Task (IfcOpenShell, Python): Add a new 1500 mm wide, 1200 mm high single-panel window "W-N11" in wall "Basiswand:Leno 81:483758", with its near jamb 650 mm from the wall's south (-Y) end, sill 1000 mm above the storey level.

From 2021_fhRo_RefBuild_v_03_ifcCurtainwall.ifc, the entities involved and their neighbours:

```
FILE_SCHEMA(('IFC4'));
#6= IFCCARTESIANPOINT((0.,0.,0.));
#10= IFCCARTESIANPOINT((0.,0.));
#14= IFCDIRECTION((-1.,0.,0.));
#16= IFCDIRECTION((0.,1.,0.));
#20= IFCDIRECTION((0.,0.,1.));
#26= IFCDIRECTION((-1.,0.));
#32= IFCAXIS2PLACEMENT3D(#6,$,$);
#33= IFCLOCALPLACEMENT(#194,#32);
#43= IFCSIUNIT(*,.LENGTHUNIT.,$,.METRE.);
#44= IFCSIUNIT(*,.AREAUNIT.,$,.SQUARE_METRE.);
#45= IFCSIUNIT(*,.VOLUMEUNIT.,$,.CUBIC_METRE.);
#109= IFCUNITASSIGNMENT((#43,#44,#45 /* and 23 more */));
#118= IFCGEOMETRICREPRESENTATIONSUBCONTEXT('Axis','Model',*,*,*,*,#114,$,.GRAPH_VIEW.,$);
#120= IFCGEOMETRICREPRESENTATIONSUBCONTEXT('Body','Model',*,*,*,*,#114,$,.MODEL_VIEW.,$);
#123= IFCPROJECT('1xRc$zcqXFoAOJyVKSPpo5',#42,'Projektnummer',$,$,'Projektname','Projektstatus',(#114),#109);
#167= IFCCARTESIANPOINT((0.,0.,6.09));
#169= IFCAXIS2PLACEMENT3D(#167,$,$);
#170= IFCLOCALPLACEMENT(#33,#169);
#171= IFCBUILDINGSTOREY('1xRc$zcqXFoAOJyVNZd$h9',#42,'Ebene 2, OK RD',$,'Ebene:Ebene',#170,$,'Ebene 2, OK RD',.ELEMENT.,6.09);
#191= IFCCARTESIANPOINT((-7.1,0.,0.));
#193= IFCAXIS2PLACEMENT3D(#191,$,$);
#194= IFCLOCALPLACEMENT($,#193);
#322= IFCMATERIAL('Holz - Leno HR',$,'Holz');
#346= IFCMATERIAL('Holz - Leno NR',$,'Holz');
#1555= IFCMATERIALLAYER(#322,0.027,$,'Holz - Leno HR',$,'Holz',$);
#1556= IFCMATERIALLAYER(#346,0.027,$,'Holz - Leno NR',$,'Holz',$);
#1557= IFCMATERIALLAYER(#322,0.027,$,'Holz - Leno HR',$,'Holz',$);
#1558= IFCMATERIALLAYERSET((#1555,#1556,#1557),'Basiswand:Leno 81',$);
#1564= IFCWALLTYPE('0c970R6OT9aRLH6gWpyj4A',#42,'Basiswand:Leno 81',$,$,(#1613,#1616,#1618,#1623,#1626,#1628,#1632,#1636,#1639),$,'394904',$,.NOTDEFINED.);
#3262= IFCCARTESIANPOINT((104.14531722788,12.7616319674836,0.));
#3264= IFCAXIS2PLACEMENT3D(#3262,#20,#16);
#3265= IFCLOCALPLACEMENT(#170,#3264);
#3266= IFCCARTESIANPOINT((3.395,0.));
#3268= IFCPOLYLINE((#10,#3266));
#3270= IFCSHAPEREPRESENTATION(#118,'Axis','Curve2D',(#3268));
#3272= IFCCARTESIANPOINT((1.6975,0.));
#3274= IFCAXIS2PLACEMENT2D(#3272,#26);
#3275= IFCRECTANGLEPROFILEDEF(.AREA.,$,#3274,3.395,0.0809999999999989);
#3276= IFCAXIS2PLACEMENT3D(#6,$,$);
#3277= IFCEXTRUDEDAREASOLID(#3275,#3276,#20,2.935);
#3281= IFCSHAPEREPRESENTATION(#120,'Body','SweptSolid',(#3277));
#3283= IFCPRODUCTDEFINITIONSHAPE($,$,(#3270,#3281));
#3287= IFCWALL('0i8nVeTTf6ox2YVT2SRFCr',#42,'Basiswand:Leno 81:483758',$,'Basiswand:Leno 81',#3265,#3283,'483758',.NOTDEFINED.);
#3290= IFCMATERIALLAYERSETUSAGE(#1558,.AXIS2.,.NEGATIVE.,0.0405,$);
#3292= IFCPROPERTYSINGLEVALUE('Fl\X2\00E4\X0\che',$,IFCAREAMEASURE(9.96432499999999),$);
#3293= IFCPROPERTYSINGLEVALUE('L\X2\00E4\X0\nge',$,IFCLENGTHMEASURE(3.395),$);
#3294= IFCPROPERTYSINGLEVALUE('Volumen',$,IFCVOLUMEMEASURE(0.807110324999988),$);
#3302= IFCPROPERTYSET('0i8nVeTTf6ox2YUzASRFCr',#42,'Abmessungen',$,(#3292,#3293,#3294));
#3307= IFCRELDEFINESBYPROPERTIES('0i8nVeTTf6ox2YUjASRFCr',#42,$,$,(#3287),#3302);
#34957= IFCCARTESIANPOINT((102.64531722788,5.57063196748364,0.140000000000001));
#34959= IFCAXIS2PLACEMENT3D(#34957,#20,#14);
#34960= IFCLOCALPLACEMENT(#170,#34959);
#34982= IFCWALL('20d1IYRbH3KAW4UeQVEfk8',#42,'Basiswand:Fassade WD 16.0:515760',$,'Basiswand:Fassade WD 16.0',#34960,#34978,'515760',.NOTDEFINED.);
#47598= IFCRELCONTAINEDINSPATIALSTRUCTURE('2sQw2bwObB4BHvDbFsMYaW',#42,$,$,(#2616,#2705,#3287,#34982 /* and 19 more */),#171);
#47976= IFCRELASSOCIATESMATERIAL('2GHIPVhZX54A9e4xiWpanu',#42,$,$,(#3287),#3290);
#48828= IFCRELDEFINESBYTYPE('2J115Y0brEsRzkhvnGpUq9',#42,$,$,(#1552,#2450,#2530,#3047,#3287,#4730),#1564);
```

```python
import numpy as np
import ifcopenshell
import ifcopenshell.api.feature
import ifcopenshell.api.geometry
import ifcopenshell.api.pset
import ifcopenshell.api.root
import ifcopenshell.api.spatial
import ifcopenshell.geom
import ifcopenshell.util.element
import ifcopenshell.util.placement
import ifcopenshell.util.representation
import ifcopenshell.util.shape
import ifcopenshell.util.unit

model = ifcopenshell.open("2021_fhRo_RefBuild_v_03_ifcCurtainwall.ifc")
unit_scale = ifcopenshell.util.unit.calculate_unit_scale(model)
area_scale = ifcopenshell.util.unit.calculate_unit_scale(model, "AREAUNIT")
volume_scale = ifcopenshell.util.unit.calculate_unit_scale(model, "VOLUMEUNIT")
settings = ifcopenshell.geom.settings()


def volume(element):
    """Net volume in cubic metres, openings subtracted."""
    shape = ifcopenshell.geom.create_shape(settings, element)
    return ifcopenshell.util.shape.get_volume(shape.geometry)


wall = model.by_id(3287)
storey = ifcopenshell.util.element.get_container(wall, ifc_class="IfcBuildingStorey")
context = ifcopenshell.util.representation.get_context(model, "Model", "Body", "MODEL_VIEW")
before = volume(wall)

width, height, from_end, sill = 1.5, 1.2, 0.65, 1  # metres

# The wall runs along its own X axis, and the end named is its -X end.
wall_shape = ifcopenshell.geom.create_shape(settings, wall)
x, y, z = ifcopenshell.util.shape.get_vertices(wall_shape.geometry).T
start = x.min() + from_end
face, thickness = float(y.min()), float(y.max() - y.min())
wall_matrix = ifcopenshell.util.placement.get_local_placement(wall.ObjectPlacement)
level = ifcopenshell.util.placement.get_local_placement(storey.ObjectPlacement)[2, 3]


def in_wall(x, y):
    """Placement at x, y metres in the wall's axes, at sill height."""
    matrix = wall_matrix.copy()
    matrix[:, 3] = wall_matrix @ np.array([x / unit_scale, y / unit_scale, 0.0, 1.0])
    matrix[2, 3] = level + sill / unit_scale
    return matrix


# Opening: a box that overshoots both wall faces by 50 mm.
opening = ifcopenshell.api.root.create_entity(model, ifc_class="IfcOpeningElement", predefined_type="OPENING")
box = ifcopenshell.api.geometry.add_wall_representation(
    model, context=context, length=width, height=height, thickness=thickness + 0.1
)
ifcopenshell.api.geometry.assign_representation(model, product=opening, representation=box)
ifcopenshell.api.geometry.edit_object_placement(model, product=opening, matrix=in_wall(start, face - 0.05), is_si=False)
ifcopenshell.api.feature.add_feature(model, feature=opening, element=wall)

window = ifcopenshell.api.root.create_entity(model, ifc_class="IfcWindow", name="W-N11", predefined_type="WINDOW")
window.OverallWidth, window.OverallHeight = width / unit_scale, height / unit_scale
window.PartitioningType = "SINGLE_PANEL"
body = ifcopenshell.api.geometry.add_window_representation(
    model,
    context=context,
    overall_width=window.OverallWidth,
    overall_height=window.OverallHeight,
    partition_type="SINGLE_PANEL",
)
ifcopenshell.api.geometry.assign_representation(model, product=window, representation=body)
ifcopenshell.api.spatial.assign_container(model, products=[window], relating_structure=storey)
ifcopenshell.api.feature.add_filling(model, opening=opening, element=window)

# Centre the window in the wall's thickness.
ifcopenshell.api.geometry.edit_object_placement(model, product=window, matrix=in_wall(start, face), is_si=False)
window_shape = ifcopenshell.geom.create_shape(settings, window)
depth = ifcopenshell.util.shape.get_vertices(window_shape.geometry)[:, 1]
offset = face + thickness / 2 - (depth.min() + depth.max()) / 2
ifcopenshell.api.geometry.edit_object_placement(model, product=window, matrix=in_wall(start, offset), is_si=False)

after = volume(wall)

# Update the wall's stored quantities.
pset = model.by_id(ifcopenshell.util.element.get_pset(wall, "Abmessungen", should_inherit=False)["id"])
ifcopenshell.api.pset.edit_pset(model, pset=pset, properties={
    "Fläche": model.create_entity("IfcAreaMeasure", after / thickness / area_scale),
    "Volumen": model.create_entity("IfcVolumeMeasure", after / volume_scale),
})

print(f"wall volume {before:.3f} -> {after:.3f} m3")

model.write("2021_fhRo_RefBuild_v_03_ifcCurtainwall_rev.ifc")
```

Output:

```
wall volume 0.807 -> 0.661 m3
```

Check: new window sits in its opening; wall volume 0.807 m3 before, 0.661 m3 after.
